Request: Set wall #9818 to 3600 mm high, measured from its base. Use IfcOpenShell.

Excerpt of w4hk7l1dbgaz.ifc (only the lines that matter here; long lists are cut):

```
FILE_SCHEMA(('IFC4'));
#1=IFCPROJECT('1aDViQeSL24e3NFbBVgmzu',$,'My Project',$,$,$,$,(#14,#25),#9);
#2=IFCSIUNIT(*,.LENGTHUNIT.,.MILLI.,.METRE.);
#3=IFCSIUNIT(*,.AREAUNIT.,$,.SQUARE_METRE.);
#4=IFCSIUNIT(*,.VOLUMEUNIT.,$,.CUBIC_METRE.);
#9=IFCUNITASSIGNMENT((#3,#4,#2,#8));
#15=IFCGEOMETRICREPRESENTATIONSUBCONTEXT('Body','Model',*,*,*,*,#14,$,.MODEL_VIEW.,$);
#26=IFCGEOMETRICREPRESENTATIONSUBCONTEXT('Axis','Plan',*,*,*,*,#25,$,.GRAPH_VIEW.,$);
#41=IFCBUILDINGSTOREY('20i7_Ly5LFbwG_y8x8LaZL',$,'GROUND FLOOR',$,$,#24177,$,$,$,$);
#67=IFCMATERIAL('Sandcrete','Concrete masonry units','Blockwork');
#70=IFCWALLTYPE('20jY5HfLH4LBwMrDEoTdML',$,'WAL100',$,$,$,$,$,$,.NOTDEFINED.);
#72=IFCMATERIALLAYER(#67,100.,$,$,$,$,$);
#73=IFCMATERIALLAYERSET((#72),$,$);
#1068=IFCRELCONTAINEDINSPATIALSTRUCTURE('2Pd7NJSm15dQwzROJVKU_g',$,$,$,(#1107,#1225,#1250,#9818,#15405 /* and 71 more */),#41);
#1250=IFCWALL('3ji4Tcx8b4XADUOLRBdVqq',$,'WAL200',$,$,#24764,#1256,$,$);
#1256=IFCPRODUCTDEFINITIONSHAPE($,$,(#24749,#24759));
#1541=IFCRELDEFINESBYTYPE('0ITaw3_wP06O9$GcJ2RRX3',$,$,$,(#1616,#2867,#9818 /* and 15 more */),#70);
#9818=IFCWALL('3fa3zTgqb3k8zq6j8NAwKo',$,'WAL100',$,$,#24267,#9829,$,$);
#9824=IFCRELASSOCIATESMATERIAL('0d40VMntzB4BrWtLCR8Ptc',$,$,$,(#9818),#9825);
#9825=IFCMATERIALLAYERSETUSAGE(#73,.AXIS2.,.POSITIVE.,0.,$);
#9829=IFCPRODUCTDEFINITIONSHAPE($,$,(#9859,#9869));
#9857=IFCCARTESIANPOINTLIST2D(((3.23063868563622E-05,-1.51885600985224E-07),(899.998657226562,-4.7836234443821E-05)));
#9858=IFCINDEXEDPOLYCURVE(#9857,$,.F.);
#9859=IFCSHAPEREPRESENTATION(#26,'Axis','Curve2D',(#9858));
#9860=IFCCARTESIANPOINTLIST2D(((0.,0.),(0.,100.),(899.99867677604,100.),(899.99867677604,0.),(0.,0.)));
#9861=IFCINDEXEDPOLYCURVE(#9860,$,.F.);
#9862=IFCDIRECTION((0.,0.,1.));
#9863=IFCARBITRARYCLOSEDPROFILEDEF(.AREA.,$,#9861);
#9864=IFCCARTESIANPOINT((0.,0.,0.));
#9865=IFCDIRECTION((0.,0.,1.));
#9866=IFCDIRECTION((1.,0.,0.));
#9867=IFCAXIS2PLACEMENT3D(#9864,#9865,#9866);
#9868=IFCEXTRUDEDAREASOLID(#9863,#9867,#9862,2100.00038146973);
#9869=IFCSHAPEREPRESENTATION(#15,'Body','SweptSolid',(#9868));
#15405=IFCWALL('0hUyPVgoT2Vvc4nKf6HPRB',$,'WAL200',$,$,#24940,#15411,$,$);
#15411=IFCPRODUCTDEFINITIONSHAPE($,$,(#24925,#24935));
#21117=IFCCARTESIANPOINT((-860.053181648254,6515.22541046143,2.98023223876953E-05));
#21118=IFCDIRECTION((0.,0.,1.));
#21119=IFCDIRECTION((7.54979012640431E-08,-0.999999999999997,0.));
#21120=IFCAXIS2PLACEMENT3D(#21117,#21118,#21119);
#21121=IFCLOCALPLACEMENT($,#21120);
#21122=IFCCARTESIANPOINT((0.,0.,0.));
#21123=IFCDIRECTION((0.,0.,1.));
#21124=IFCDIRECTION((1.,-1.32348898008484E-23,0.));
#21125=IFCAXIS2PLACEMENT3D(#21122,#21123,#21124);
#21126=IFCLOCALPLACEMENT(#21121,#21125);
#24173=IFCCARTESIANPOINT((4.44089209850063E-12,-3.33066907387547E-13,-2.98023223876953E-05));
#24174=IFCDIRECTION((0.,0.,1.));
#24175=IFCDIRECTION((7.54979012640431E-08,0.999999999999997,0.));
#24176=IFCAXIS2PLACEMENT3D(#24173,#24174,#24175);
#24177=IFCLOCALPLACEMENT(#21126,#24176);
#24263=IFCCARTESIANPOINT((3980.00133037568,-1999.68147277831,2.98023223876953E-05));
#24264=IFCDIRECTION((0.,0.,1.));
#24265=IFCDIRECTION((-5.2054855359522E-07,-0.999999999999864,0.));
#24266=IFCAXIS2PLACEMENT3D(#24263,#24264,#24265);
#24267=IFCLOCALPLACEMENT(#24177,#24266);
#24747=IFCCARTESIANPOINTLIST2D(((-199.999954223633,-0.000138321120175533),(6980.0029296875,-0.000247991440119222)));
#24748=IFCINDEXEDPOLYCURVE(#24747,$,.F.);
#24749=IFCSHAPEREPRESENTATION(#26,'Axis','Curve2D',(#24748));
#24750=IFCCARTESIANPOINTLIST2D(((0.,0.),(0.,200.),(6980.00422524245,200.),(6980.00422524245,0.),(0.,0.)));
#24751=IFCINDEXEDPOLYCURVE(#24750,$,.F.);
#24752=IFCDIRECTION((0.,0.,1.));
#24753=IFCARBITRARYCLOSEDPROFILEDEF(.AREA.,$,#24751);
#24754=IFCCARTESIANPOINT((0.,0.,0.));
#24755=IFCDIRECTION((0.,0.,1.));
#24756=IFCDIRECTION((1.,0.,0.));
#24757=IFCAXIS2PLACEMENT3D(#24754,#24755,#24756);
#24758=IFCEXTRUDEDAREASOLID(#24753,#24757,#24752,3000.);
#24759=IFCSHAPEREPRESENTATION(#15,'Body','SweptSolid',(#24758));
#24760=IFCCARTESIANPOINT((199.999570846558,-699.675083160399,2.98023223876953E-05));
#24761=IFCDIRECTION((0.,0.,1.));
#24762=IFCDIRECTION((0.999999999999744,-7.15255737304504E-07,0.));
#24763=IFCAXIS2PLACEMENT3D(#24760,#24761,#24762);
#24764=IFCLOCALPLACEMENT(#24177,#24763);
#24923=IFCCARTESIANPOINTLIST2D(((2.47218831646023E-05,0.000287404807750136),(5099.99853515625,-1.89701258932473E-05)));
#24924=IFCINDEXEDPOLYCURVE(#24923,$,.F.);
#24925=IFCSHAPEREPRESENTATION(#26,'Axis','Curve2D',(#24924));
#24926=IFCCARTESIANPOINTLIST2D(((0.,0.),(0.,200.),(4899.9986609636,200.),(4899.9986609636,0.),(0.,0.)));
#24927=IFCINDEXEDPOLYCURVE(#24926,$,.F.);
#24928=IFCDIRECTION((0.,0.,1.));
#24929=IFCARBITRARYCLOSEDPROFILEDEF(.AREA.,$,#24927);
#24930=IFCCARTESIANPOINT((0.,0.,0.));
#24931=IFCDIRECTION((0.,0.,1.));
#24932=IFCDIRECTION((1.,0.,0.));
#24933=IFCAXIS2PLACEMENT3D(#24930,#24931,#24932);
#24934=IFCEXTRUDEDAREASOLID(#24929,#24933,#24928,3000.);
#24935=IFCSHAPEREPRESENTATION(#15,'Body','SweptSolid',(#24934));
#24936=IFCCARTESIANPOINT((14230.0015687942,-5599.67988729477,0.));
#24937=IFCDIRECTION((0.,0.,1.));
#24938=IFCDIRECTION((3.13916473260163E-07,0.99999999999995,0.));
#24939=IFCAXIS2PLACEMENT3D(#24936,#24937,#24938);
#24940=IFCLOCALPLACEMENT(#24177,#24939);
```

```python
import ifcopenshell
import ifcopenshell.geom
import ifcopenshell.util.representation
import ifcopenshell.util.shape

model = ifcopenshell.open("w4hk7l1dbgaz.ifc")
settings = ifcopenshell.geom.settings()


def volume(element):
    """Net volume in cubic metres, openings subtracted."""
    shape = ifcopenshell.geom.create_shape(settings, element)
    return ifcopenshell.util.shape.get_volume(shape.geometry)


wall = model.by_guid("3fa3zTgqb3k8zq6j8NAwKo")
before = volume(wall)

body = ifcopenshell.util.representation.get_representation(wall, "Model", "Body")
solid = body.Items[0]
old_height = solid.Depth
solid.Depth = 3600.0
after = volume(wall)

print(f"height {old_height:g} -> {solid.Depth:g}, volume {before:.3f} -> {after:.3f} m3")

model.write("w4hk7l1dbgaz-out.ifc")
```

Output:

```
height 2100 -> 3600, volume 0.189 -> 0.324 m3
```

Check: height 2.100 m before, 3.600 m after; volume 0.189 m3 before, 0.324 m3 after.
